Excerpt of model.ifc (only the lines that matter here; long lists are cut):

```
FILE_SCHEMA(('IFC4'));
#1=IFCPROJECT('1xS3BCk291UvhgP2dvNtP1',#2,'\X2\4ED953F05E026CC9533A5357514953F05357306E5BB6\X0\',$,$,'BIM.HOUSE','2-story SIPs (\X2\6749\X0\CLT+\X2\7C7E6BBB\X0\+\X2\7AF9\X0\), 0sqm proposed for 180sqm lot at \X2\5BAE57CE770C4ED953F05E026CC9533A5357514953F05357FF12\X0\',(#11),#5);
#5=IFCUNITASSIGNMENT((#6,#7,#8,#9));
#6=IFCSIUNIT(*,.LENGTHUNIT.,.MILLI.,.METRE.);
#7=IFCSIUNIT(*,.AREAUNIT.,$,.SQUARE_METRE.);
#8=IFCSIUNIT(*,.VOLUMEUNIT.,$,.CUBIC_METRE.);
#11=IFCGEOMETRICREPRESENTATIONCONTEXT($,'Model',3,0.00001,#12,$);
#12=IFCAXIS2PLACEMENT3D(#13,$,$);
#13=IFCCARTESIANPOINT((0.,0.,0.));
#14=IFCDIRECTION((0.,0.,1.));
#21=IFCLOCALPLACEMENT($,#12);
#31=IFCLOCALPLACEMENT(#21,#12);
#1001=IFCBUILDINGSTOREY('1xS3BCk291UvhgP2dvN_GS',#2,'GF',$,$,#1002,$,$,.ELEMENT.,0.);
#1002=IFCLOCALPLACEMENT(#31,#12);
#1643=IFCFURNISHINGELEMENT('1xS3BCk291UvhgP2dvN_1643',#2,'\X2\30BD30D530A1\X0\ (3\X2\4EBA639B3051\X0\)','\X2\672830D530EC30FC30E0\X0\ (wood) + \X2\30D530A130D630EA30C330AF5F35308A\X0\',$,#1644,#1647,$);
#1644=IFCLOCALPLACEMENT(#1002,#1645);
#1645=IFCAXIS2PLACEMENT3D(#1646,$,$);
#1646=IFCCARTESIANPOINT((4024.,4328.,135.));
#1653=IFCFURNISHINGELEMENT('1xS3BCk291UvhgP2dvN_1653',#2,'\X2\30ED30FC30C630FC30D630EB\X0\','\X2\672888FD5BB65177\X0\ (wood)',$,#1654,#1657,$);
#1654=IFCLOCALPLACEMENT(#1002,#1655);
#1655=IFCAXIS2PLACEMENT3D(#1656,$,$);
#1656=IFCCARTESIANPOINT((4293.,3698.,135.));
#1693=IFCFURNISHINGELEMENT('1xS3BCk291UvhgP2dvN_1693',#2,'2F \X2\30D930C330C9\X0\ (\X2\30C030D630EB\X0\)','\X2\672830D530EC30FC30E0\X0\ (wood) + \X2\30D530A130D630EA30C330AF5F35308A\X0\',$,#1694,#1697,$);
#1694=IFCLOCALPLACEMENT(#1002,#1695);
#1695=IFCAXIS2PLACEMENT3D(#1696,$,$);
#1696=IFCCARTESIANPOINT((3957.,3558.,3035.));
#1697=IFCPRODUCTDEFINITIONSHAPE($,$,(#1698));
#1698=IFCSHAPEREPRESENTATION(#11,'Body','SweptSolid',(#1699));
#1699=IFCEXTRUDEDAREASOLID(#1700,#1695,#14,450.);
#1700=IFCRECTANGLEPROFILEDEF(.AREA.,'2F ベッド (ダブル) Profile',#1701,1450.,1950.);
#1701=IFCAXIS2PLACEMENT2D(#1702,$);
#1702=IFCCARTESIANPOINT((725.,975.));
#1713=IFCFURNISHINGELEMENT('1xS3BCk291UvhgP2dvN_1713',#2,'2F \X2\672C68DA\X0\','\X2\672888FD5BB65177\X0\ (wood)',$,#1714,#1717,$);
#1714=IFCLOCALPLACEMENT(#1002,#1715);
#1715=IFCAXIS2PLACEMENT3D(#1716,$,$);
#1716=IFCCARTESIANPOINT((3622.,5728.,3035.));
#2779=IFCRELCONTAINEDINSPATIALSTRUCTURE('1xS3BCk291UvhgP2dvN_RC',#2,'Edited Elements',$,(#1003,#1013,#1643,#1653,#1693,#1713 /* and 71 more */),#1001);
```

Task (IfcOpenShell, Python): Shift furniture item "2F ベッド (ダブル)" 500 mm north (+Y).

```python
import ifcopenshell
import ifcopenshell.api.geometry
import ifcopenshell.util.placement
import ifcopenshell.util.unit

model = ifcopenshell.open("model.ifc")
unit_scale = ifcopenshell.util.unit.calculate_unit_scale(model)

item = model.by_guid("1xS3BCk291UvhgP2dvN_1693")
matrix = ifcopenshell.util.placement.get_local_placement(item.ObjectPlacement)
matrix[1, 3] += 0.5 / unit_scale
ifcopenshell.api.geometry.edit_object_placement(model, product=item, matrix=matrix, is_si=False)

print(ifcopenshell.util.placement.get_local_placement(item.ObjectPlacement).round(3) + 0.0)

model.write("model_v2.ifc")
```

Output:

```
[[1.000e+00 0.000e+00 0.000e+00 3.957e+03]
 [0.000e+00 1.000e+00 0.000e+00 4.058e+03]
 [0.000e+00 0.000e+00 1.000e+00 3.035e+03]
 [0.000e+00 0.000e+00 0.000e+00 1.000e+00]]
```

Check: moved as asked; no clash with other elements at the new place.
